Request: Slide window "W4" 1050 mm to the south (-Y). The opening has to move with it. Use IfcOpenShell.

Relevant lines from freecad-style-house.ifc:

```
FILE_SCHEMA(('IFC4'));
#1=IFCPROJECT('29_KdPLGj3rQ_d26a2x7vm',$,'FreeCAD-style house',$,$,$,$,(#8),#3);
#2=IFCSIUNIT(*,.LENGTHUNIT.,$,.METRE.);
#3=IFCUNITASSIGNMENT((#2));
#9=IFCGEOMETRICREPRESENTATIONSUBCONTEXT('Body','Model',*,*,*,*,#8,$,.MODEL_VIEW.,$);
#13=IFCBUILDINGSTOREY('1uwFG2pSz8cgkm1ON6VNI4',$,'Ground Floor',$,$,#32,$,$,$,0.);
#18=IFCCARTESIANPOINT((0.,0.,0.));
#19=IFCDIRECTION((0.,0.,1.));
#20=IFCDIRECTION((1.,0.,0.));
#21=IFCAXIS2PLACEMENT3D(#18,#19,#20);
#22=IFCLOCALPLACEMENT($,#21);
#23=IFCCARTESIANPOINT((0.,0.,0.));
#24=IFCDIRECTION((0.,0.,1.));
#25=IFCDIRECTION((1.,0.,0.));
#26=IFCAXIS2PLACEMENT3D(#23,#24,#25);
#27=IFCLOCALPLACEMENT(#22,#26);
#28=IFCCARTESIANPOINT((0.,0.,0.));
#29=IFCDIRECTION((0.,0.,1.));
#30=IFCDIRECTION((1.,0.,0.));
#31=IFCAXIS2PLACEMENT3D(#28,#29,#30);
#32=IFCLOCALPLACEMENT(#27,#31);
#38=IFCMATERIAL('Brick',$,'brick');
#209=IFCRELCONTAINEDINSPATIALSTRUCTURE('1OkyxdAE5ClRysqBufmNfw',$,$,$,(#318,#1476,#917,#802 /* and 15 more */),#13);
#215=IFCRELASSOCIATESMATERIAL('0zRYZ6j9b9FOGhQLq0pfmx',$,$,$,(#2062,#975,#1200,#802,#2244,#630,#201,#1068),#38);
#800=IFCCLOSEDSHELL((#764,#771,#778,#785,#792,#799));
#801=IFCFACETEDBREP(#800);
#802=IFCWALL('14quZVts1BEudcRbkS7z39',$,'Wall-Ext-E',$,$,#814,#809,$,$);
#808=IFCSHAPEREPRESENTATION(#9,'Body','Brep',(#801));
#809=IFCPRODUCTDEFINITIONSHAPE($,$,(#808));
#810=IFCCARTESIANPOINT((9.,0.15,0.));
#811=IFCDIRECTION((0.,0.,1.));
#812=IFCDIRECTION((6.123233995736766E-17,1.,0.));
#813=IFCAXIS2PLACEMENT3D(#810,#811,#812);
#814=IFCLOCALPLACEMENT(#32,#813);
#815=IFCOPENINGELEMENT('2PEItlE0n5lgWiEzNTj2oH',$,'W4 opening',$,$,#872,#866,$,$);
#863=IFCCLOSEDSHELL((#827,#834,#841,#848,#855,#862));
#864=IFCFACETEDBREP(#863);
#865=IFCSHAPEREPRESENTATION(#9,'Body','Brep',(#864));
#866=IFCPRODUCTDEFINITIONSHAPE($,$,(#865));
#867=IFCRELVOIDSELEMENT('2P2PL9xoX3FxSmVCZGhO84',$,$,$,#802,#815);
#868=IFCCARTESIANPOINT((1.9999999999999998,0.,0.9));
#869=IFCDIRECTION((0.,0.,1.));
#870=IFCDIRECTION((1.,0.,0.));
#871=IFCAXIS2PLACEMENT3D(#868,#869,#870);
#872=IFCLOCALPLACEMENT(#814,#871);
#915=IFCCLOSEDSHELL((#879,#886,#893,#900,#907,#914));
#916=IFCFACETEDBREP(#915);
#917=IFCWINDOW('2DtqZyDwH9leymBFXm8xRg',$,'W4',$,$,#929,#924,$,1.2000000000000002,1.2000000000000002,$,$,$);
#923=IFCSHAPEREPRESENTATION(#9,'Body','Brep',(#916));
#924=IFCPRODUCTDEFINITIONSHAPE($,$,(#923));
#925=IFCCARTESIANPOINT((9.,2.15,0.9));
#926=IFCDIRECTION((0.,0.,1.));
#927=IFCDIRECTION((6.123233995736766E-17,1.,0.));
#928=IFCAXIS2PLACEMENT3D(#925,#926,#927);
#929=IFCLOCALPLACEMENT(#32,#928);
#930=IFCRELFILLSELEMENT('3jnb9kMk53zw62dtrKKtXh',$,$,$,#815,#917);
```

```python
import ifcopenshell
import ifcopenshell.api.geometry
import ifcopenshell.util.placement
import ifcopenshell.util.unit

model = ifcopenshell.open("freecad-style-house.ifc")
unit_scale = ifcopenshell.util.unit.calculate_unit_scale(model)

window = model.by_guid("2DtqZyDwH9leymBFXm8xRg")
opening = window.FillsVoids[0].RelatingOpeningElement
wall = opening.VoidsElements[0].RelatingBuildingElement

wall_matrix = ifcopenshell.util.placement.get_local_placement(wall.ObjectPlacement)
shift = wall_matrix[:3, 0] * -1.05 / unit_scale
before = ifcopenshell.util.placement.get_local_placement(window.ObjectPlacement)[:3, 3].copy()

# The window is not placed relative to its opening, so move both.
for product in (opening, window):
    matrix = ifcopenshell.util.placement.get_local_placement(product.ObjectPlacement)
    matrix[:3, 3] += shift
    ifcopenshell.api.geometry.edit_object_placement(model, product=product, matrix=matrix, is_si=False)

after = ifcopenshell.util.placement.get_local_placement(window.ObjectPlacement)[:3, 3]
print("window moved by", (after - before).round(3) + 0.0)

model.write("freecad-style-house_updated.ifc")
```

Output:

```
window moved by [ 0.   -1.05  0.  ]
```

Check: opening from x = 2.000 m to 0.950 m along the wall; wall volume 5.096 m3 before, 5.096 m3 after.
